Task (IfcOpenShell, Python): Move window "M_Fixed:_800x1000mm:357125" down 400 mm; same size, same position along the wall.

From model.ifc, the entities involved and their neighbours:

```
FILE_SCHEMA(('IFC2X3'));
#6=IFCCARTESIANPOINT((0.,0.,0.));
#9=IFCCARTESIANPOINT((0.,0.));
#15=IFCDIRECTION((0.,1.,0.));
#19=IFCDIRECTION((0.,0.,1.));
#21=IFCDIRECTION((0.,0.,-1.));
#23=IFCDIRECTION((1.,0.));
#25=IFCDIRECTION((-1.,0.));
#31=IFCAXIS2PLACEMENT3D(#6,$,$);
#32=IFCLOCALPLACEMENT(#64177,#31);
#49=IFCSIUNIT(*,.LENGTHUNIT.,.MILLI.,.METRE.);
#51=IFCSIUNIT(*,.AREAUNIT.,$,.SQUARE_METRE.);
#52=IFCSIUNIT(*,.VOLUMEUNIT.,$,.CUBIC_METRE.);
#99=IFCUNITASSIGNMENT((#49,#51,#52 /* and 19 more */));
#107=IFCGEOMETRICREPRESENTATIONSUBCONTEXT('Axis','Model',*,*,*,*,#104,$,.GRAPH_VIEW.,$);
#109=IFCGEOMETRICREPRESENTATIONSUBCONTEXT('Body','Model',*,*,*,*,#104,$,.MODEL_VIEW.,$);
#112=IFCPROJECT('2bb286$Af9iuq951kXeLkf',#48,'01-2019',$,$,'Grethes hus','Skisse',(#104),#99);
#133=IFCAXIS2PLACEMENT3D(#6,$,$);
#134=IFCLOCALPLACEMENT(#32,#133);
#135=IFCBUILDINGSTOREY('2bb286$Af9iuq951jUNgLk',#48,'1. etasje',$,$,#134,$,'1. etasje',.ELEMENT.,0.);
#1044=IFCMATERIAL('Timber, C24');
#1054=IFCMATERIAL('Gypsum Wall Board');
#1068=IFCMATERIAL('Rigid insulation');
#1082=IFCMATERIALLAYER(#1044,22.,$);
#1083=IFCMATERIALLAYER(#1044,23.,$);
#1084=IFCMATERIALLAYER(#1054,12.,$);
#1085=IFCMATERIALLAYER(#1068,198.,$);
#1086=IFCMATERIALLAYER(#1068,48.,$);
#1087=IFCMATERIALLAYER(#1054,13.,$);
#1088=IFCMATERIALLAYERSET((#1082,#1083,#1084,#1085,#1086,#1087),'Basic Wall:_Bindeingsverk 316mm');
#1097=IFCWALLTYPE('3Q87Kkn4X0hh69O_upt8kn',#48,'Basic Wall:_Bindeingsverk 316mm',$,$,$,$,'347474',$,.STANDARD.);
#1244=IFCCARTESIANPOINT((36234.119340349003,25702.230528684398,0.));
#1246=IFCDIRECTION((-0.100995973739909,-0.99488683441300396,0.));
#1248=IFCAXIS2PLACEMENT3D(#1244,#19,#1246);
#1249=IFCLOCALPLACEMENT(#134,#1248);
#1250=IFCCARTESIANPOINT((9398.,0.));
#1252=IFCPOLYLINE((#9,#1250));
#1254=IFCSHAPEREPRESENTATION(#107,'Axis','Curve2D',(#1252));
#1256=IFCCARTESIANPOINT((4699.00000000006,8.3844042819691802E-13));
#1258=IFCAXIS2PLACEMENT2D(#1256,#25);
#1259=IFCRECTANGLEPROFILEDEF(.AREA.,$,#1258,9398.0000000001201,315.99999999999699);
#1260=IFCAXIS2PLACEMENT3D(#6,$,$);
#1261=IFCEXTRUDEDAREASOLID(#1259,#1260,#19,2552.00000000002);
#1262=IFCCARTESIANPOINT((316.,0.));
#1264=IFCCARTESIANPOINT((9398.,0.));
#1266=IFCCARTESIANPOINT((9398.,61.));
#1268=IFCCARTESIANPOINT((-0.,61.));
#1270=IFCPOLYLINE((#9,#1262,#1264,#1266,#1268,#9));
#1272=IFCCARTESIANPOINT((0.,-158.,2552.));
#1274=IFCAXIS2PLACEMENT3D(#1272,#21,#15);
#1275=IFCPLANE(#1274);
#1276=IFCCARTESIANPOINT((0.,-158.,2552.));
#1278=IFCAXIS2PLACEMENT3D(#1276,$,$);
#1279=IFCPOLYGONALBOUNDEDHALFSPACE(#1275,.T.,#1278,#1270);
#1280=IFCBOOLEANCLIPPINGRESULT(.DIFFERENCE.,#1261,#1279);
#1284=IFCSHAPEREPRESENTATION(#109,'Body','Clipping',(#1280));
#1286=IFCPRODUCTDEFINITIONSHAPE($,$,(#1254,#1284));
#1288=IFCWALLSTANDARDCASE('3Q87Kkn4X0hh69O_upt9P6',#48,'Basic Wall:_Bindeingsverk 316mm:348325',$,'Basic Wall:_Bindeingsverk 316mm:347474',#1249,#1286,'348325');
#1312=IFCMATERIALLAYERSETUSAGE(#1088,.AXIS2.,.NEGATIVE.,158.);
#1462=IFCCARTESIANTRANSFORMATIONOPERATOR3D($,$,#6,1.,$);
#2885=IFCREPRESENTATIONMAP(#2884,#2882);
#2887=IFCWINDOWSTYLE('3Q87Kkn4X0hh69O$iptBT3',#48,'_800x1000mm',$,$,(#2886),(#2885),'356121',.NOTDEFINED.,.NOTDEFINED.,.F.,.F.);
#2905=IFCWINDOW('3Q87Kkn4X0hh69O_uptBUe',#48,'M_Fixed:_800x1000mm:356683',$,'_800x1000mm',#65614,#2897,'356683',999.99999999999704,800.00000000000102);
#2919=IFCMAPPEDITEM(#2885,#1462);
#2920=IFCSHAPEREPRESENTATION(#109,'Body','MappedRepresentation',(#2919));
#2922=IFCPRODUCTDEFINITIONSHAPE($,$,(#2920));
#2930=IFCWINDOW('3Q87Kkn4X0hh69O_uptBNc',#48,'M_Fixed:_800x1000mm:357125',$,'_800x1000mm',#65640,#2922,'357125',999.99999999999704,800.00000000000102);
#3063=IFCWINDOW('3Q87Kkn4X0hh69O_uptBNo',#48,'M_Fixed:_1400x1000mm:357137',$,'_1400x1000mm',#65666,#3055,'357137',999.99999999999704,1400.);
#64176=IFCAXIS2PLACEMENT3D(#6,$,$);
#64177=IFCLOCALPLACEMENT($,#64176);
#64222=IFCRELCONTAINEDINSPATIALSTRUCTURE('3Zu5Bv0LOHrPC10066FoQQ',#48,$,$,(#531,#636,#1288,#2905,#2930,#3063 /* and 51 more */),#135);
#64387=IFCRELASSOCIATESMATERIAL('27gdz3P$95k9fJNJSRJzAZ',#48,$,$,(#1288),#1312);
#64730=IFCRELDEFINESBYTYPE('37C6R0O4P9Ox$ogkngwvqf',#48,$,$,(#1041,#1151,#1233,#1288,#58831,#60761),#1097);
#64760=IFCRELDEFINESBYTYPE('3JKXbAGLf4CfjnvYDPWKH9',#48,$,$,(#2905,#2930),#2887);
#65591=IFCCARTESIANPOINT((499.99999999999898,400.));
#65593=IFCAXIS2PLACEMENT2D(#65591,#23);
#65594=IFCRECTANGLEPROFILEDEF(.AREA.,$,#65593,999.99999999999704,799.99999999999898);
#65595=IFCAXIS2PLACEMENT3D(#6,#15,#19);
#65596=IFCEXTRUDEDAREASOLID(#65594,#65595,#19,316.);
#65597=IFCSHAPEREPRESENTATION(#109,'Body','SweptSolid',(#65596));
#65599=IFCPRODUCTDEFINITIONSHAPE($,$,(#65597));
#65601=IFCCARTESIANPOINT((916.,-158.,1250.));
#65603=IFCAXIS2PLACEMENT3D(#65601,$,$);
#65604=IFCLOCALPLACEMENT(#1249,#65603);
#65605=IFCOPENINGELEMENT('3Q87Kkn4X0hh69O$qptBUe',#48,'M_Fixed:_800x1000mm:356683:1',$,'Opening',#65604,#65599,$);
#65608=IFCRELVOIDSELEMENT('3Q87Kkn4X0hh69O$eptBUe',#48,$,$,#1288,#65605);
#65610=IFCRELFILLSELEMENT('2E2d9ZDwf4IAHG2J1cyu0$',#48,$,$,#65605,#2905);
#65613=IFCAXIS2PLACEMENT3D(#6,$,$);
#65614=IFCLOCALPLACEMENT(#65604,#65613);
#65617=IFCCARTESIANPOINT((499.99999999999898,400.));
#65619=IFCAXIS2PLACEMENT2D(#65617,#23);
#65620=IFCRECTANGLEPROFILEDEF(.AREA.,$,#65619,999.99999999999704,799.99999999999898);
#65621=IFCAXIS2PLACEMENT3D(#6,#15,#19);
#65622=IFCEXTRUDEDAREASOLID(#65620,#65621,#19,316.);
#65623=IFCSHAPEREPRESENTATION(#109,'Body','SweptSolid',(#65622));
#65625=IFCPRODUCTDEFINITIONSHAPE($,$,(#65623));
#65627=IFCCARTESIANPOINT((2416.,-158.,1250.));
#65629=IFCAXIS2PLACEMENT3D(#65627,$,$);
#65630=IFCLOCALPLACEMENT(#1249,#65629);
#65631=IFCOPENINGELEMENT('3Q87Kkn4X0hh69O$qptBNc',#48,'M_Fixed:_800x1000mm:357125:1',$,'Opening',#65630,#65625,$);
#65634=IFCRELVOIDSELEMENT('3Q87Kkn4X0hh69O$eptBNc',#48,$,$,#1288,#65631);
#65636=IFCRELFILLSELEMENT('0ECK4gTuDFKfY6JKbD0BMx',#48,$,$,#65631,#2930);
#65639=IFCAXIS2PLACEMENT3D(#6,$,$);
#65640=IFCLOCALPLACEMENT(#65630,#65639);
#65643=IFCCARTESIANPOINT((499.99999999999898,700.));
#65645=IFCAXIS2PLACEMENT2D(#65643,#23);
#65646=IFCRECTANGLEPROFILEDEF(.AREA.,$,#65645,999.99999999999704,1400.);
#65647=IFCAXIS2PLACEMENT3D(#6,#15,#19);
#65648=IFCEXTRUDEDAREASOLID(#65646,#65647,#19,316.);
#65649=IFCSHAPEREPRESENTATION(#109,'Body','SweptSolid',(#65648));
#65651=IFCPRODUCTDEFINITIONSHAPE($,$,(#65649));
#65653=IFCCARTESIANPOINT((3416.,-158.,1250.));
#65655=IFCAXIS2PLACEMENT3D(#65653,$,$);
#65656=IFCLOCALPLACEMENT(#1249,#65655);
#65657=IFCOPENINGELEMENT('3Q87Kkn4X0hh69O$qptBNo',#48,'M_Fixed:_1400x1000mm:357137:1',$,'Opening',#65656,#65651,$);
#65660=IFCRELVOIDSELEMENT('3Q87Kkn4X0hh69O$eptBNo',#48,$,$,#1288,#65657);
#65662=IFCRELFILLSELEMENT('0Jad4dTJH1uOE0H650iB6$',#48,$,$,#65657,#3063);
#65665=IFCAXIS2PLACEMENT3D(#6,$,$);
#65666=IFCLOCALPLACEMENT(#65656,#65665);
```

```python
import numpy as np
import ifcopenshell
import ifcopenshell.api.geometry
import ifcopenshell.util.placement
import ifcopenshell.util.unit

model = ifcopenshell.open("model.ifc")
unit_scale = ifcopenshell.util.unit.calculate_unit_scale(model)

window = model.by_id(2930)
opening = window.FillsVoids[0].RelatingOpeningElement
dz = -0.4 / unit_scale

shift = np.array([0.0, 0.0, dz])
# The window is placed relative to its opening, so it follows when the opening moves.
matrix = ifcopenshell.util.placement.get_local_placement(opening.ObjectPlacement)
matrix[:3, 3] += shift
ifcopenshell.api.geometry.edit_object_placement(
    model, product=opening, matrix=matrix, is_si=False, should_transform_children=True
)

print(f"moved by {dz * unit_scale:+.3f} m")

model.write("model_edited.ifc")
```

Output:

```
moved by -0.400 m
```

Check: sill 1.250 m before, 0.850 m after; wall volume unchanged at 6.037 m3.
